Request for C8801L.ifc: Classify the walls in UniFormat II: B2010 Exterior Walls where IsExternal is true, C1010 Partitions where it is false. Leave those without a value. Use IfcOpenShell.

First a look at what the model holds.

```python
import ifcopenshell
import ifcopenshell.util.element

model = ifcopenshell.open("C8801L.ifc")
print(model.schema)
print("classifications:", [c.Name for c in model.by_type("IfcClassification")])
values = [ifcopenshell.util.element.get_pset(e, "Pset_WallCommon", "IsExternal") for e in model.by_type("IfcWall")]
for value in (True, False, None):
    print("IsExternal", value, values.count(value))
```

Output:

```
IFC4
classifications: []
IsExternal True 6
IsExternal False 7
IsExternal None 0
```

```python
import ifcopenshell
import ifcopenshell.api.classification
import ifcopenshell.util.element

model = ifcopenshell.open("C8801L.ifc")

system = ifcopenshell.api.classification.add_classification(model, classification="UniFormat II")

walls = model.by_type("IfcWall")
external = {e: ifcopenshell.util.element.get_pset(e, "Pset_WallCommon", "IsExternal") for e in walls}
for flag, code, name in ((True, "B2010", "Exterior Walls"), (False, "C1010", "Partitions")):
    products = [e for e in walls if external[e] is flag]
    ifcopenshell.api.classification.add_reference(
        model, products=products, classification=system, identification=code, name=name
    )
    print(code, len(products))

model.write("C8801L_updated.ifc")
```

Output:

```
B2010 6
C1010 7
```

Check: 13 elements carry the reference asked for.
